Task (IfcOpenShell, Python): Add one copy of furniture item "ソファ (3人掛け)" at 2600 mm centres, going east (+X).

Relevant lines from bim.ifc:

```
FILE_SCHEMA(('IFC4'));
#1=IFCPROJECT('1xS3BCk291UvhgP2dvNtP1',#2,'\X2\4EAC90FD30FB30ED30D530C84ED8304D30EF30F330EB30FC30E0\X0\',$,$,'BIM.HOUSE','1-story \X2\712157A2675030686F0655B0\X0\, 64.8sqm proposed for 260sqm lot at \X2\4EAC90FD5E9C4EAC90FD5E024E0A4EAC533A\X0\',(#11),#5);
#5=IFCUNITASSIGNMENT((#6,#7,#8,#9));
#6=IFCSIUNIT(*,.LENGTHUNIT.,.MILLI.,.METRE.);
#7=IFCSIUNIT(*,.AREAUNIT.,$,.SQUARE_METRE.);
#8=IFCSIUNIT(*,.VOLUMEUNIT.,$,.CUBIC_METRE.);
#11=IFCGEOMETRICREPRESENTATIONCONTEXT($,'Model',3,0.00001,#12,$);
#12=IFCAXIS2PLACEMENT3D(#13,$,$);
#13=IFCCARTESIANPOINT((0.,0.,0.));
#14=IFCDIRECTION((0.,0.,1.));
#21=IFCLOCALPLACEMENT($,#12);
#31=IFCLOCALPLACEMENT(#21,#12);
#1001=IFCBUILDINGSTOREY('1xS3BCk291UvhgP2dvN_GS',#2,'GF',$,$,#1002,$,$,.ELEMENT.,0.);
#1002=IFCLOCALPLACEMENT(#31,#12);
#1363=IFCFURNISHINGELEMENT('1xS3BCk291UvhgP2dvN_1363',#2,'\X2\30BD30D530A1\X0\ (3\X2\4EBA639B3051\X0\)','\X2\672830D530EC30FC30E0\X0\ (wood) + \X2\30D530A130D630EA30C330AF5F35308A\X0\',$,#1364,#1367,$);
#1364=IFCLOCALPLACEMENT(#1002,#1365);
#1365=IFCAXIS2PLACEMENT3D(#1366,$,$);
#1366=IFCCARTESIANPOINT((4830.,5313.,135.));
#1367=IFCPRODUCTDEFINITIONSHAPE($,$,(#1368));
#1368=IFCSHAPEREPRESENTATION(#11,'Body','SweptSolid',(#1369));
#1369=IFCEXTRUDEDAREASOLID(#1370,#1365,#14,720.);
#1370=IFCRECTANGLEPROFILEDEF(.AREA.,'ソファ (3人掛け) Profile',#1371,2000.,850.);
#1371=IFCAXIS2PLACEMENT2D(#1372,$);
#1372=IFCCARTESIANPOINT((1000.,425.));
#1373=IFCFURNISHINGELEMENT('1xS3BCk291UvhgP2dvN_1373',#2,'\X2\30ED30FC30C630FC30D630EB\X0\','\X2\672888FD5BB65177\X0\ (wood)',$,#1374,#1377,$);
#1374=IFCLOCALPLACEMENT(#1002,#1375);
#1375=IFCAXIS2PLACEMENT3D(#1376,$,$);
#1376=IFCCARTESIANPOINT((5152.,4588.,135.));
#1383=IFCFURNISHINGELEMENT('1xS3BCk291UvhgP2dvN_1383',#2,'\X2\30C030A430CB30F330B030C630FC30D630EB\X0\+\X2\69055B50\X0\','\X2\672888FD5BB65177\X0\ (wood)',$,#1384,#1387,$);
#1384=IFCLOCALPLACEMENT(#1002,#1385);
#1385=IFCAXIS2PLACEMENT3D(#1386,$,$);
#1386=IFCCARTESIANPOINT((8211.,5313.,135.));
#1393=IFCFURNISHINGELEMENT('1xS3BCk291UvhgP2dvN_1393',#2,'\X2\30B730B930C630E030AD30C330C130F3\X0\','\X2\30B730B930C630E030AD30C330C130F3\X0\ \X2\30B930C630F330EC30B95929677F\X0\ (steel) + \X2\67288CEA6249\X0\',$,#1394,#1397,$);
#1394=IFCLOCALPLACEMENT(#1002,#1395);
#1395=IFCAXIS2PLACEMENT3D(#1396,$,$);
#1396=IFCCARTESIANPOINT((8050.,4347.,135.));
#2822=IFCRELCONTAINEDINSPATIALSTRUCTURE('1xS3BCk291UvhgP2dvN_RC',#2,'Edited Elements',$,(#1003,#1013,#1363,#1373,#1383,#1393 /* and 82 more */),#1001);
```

```python
import numpy as np
import ifcopenshell
import ifcopenshell.api.geometry
import ifcopenshell.api.root
import ifcopenshell.util.element
import ifcopenshell.util.placement
import ifcopenshell.util.unit

model = ifcopenshell.open("bim.ifc")
unit_scale = ifcopenshell.util.unit.calculate_unit_scale(model)


def reuse_history(source, copy):
    """copy_class also copies each property set's owner history, people and application; keep the originals."""
    for rel in copy.IsDefinedBy:
        if rel.is_a("IfcRelDefinesByProperties") and (history := rel.RelatingPropertyDefinition.OwnerHistory):
            rel.RelatingPropertyDefinition.OwnerHistory = source.OwnerHistory
            ifcopenshell.util.element.remove_deep2(model, history)


source = model.by_guid("1xS3BCk291UvhgP2dvN_1363")
base = ifcopenshell.util.placement.get_local_placement(source.ObjectPlacement)
step = np.array([1.0, 0.0, 0.0]) * 2.6 / unit_scale

for i in range(1, 2):
    copy = ifcopenshell.api.root.copy_class(model, product=source)
    copy.Representation = ifcopenshell.util.element.copy_deep(
        model, source.Representation, exclude=["IfcGeometricRepresentationContext", "IfcRepresentationMap"]
    )
    reuse_history(source, copy)
    matrix = base.copy()
    matrix[:3, 3] += i * step
    print("added at", matrix[:3, 3].round(3) + 0.0)
    ifcopenshell.api.geometry.edit_object_placement(model, product=copy, matrix=matrix, is_si=False)

model.write("bim_rev.ifc")
```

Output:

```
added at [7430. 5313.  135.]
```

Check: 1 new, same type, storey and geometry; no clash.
